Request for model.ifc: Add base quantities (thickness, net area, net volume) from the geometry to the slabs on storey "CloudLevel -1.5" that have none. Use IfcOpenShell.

First a look at what the model holds.

```python
import ifcopenshell
import ifcopenshell.util.element
import ifcopenshell.util.unit

model = ifcopenshell.open("model.ifc")
print(model.schema)
for unit_type in ("LENGTHUNIT", "AREAUNIT", "VOLUMEUNIT"):
    print(unit_type, ifcopenshell.util.unit.calculate_unit_scale(model, unit_type))
storey = next(s for s in model.by_type("IfcBuildingStorey") if s.Name == "CloudLevel -1.5")
slabs = [e for e in ifcopenshell.util.element.get_decomposition(storey) if e.is_a("IfcSlab")]
for e in sorted(slabs, key=lambda e: e.id()):
    print(e.id(), e.is_a(), e.Name, list(ifcopenshell.util.element.get_psets(e, qtos_only=True)), sep=" | ")
```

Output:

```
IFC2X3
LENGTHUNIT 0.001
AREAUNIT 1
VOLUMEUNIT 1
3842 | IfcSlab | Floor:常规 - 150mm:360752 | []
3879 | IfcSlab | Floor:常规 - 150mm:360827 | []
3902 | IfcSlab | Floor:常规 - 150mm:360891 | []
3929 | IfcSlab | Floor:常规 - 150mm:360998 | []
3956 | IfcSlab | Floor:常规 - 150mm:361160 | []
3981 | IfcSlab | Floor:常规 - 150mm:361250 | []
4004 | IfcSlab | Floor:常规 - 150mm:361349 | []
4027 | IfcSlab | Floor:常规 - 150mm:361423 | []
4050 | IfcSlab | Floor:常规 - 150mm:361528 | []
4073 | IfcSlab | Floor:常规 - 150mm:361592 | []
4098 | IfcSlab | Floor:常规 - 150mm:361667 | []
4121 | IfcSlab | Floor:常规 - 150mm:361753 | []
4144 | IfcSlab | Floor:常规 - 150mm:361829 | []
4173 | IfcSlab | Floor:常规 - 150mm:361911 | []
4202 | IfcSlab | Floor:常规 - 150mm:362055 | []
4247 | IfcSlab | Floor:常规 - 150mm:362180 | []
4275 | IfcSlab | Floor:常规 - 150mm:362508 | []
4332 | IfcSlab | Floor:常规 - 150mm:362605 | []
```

```python
import ifcopenshell
import ifcopenshell.api.pset
import ifcopenshell.geom
import ifcopenshell.util.element
import ifcopenshell.util.shape
import ifcopenshell.util.unit

model = ifcopenshell.open("model.ifc")
unit_scale = ifcopenshell.util.unit.calculate_unit_scale(model)
area_scale = ifcopenshell.util.unit.calculate_unit_scale(model, "AREAUNIT")
volume_scale = ifcopenshell.util.unit.calculate_unit_scale(model, "VOLUMEUNIT")
settings = ifcopenshell.geom.settings()

storey = next(s for s in model.by_type("IfcBuildingStorey") if s.Name == "CloudLevel -1.5")
slabs = [e for e in ifcopenshell.util.element.get_decomposition(storey) if e.is_a("IfcSlab")]

for e in sorted(slabs, key=lambda e: e.id()):
    if ifcopenshell.util.element.get_psets(e, qtos_only=True, should_inherit=False):
        continue
    # Geometry comes back in metres, in the element's own axes.
    shape = ifcopenshell.geom.create_shape(settings, e)
    values = {
        "Width": ifcopenshell.util.shape.get_z(shape.geometry) / unit_scale,
        "NetArea": ifcopenshell.util.shape.get_footprint_area(shape.geometry) / area_scale,
        "NetVolume": ifcopenshell.util.shape.get_volume(shape.geometry) / volume_scale,
    }
    qto = ifcopenshell.api.pset.add_qto(model, product=e, name="BaseQuantities")
    ifcopenshell.api.pset.edit_qto(model, qto=qto, properties=values)
    print(e.id(), {k: round(v, 3) for k, v in values.items()})

model.write("model_edited.ifc")
```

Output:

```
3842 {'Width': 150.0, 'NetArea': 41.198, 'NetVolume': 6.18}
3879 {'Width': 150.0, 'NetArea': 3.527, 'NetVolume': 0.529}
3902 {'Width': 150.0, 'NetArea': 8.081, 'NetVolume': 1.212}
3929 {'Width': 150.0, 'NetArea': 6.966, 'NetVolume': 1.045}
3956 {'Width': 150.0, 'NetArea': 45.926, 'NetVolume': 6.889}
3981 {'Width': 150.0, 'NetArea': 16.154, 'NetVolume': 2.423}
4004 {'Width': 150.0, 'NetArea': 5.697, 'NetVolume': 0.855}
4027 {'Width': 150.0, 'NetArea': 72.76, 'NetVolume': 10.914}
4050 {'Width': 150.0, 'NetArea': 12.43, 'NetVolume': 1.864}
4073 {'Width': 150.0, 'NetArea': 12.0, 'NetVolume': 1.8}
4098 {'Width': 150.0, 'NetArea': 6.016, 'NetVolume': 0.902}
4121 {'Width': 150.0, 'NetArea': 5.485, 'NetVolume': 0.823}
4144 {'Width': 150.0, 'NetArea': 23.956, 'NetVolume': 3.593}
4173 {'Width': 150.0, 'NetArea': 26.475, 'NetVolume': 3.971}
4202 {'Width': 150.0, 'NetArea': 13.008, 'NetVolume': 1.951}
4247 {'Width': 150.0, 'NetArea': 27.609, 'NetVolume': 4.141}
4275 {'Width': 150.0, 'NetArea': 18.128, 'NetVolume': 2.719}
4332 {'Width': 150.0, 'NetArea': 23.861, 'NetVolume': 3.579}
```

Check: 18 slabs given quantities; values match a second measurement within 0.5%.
